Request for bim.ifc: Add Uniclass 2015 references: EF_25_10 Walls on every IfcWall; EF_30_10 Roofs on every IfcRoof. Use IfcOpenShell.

First a look at what the model holds.

```python
import ifcopenshell

model = ifcopenshell.open("bim.ifc")
print(model.schema)
print("classifications:", [c.Name for c in model.by_type("IfcClassification")])
for ifc_class in ("IfcDoor", "IfcRoof", "IfcStair", "IfcWall", "IfcWindow"):
    print(ifc_class, len(model.by_type(ifc_class)))
```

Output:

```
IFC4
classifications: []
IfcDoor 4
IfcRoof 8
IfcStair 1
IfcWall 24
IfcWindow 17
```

```python
import ifcopenshell
import ifcopenshell.api.classification

model = ifcopenshell.open("bim.ifc")

system = ifcopenshell.api.classification.add_classification(model, classification="Uniclass 2015")

codes = {
    "IfcWall": ("EF_25_10", "Walls"),
    "IfcRoof": ("EF_30_10", "Roofs"),
}
for ifc_class, (code, name) in codes.items():
    products = model.by_type(ifc_class)
    ifcopenshell.api.classification.add_reference(
        model, products=products, classification=system, identification=code, name=name
    )
    print(code, len(products))

model.write("bim-out.ifc")
```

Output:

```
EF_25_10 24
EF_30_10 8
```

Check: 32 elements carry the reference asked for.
